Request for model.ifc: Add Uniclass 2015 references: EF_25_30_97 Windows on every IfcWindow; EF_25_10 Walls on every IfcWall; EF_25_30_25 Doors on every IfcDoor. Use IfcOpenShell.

First a look at what the model holds.

```python
import ifcopenshell

model = ifcopenshell.open("model.ifc")
print(model.schema)
print("classifications:", [c.Name for c in model.by_type("IfcClassification")])
for ifc_class in ("IfcDoor", "IfcRoof", "IfcStair", "IfcWall", "IfcWindow"):
    print(ifc_class, len(model.by_type(ifc_class)))
```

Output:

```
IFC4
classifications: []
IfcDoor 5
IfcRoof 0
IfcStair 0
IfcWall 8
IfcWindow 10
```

```python
import ifcopenshell
import ifcopenshell.api.classification

model = ifcopenshell.open("model.ifc")

system = ifcopenshell.api.classification.add_classification(model, classification="Uniclass 2015")

codes = {
    "IfcWindow": ("EF_25_30_97", "Windows"),
    "IfcWall": ("EF_25_10", "Walls"),
    "IfcDoor": ("EF_25_30_25", "Doors"),
}
for ifc_class, (code, name) in codes.items():
    products = model.by_type(ifc_class)
    ifcopenshell.api.classification.add_reference(
        model, products=products, classification=system, identification=code, name=name
    )
    print(code, len(products))

model.write("model-out.ifc")
```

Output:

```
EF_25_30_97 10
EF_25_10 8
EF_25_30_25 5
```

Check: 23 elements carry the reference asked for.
